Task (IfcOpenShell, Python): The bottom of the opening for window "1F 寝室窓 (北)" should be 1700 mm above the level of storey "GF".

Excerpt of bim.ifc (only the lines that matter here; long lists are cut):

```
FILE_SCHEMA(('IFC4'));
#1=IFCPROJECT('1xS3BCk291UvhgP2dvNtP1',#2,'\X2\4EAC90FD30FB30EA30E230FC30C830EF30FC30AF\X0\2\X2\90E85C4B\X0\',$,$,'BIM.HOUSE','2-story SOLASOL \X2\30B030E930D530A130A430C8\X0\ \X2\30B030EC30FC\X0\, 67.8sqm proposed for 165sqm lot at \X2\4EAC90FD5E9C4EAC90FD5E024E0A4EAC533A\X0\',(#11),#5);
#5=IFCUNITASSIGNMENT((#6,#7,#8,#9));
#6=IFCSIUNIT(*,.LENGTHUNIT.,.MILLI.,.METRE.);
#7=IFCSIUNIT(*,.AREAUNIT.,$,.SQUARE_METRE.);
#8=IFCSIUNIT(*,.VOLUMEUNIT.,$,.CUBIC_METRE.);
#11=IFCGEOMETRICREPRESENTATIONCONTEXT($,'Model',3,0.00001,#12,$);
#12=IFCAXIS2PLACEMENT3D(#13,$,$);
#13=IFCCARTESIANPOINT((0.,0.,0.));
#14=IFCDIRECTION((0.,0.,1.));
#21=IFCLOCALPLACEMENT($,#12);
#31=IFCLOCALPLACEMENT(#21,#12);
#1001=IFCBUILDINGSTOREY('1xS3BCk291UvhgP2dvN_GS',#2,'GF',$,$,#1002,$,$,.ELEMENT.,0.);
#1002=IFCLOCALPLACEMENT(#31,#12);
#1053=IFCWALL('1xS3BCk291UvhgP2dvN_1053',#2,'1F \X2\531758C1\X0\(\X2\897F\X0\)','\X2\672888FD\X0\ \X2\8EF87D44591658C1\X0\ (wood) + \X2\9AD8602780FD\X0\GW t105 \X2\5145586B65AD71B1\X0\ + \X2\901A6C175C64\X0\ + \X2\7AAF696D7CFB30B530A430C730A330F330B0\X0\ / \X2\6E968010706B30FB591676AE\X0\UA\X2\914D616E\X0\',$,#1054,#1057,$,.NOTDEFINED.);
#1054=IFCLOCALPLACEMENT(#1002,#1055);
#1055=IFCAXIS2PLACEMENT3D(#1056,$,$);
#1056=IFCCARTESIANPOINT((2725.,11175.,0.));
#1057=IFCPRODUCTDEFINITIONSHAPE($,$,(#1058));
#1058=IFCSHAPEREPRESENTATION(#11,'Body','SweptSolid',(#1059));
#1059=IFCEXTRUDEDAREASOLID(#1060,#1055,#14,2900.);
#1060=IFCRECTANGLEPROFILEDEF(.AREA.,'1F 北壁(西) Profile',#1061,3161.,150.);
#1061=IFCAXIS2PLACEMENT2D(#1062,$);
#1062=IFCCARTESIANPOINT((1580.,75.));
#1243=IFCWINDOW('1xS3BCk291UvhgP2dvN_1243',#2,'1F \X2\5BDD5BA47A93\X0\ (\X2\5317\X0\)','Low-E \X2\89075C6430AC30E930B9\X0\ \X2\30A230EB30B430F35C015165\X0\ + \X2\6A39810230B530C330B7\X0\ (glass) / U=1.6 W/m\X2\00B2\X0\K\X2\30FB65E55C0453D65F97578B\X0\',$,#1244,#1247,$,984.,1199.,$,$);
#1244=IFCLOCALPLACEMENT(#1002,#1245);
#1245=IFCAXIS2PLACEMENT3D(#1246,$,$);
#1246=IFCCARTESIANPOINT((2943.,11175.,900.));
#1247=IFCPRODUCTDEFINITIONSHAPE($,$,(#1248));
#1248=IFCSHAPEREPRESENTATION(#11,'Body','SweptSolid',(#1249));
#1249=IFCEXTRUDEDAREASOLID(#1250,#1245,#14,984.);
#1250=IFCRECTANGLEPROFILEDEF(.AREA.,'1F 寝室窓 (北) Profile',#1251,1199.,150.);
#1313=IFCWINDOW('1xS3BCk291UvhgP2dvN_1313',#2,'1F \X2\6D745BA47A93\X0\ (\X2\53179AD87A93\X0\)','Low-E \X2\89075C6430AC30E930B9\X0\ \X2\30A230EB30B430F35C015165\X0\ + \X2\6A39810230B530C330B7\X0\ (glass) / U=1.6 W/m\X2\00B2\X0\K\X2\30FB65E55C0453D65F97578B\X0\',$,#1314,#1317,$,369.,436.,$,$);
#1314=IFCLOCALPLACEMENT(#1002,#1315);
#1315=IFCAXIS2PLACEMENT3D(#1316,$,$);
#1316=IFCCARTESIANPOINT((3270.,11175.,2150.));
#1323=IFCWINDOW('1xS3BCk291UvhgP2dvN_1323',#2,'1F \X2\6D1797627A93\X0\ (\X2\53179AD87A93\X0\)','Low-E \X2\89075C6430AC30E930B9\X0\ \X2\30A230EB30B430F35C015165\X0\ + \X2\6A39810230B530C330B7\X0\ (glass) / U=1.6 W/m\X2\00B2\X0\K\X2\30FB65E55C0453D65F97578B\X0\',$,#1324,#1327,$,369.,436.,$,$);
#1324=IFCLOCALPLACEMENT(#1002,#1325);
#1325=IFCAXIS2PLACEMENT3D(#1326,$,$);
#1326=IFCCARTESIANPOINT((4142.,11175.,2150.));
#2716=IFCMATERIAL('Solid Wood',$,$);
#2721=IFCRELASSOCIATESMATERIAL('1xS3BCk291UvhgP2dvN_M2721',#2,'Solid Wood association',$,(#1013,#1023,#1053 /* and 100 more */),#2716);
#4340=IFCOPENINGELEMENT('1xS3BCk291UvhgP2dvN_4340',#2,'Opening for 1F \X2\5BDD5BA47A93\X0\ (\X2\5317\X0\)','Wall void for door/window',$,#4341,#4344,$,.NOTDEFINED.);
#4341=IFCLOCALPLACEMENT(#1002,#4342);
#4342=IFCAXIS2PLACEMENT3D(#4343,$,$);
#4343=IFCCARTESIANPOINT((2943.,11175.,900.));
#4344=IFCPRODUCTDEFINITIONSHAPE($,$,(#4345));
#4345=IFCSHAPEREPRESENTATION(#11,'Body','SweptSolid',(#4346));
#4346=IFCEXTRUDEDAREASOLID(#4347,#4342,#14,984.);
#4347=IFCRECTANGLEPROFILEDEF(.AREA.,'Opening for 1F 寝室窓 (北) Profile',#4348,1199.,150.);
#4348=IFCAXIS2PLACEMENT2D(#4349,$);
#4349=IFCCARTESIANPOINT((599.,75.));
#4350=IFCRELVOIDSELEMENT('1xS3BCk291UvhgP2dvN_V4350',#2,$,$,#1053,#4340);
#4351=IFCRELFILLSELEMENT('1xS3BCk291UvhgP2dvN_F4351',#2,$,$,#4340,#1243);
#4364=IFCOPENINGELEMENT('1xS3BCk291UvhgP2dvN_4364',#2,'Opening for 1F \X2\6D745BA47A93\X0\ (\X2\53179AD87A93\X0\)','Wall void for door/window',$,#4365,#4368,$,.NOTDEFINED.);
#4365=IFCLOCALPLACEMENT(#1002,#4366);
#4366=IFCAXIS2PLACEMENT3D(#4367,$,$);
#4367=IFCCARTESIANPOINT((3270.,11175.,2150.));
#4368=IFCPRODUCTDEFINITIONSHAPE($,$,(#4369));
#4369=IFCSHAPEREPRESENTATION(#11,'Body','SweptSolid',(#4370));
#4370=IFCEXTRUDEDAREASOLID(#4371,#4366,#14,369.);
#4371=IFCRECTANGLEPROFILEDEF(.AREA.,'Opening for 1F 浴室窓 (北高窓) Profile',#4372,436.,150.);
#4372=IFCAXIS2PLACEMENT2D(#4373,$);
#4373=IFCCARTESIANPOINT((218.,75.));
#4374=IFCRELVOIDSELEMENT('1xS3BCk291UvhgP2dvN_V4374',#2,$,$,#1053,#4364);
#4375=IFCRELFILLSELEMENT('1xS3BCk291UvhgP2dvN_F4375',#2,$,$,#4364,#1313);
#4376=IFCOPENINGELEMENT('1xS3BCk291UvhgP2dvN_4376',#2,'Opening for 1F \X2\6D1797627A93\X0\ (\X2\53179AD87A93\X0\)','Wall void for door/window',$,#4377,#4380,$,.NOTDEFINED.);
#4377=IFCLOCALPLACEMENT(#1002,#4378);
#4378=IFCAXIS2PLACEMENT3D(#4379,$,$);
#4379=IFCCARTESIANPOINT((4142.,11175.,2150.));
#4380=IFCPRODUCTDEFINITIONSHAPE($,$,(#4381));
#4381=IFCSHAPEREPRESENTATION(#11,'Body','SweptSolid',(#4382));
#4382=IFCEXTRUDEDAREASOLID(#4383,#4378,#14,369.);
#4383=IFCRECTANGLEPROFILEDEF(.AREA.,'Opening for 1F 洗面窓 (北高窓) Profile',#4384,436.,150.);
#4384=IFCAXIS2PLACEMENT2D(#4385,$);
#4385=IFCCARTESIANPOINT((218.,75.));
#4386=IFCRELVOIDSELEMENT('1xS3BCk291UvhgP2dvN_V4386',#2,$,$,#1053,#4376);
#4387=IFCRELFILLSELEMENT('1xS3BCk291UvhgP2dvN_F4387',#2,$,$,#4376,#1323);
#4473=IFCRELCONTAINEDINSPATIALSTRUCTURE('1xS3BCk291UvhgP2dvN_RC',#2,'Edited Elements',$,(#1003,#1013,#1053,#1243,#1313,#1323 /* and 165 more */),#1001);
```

```python
import numpy as np
import ifcopenshell
import ifcopenshell.api.geometry
import ifcopenshell.geom
import ifcopenshell.util.element
import ifcopenshell.util.placement
import ifcopenshell.util.shape
import ifcopenshell.util.unit

model = ifcopenshell.open("bim.ifc")
unit_scale = ifcopenshell.util.unit.calculate_unit_scale(model)

window = model.by_guid("1xS3BCk291UvhgP2dvN_1243")
opening = window.FillsVoids[0].RelatingOpeningElement
storey = ifcopenshell.util.element.get_container(window, ifc_class="IfcBuildingStorey")
level = ifcopenshell.util.placement.get_local_placement(storey.ObjectPlacement)[2, 3]

# The opening's origin need not be at the sill, so measure its lowest point.
shape = ifcopenshell.geom.create_shape(ifcopenshell.geom.settings(), opening)
bottom = ifcopenshell.util.shape.get_shape_bottom_elevation(shape, shape.geometry) / unit_scale
dz = level + 1.7 / unit_scale - bottom

shift = np.array([0.0, 0.0, dz])
# The window is not placed relative to its opening, so move both.
for product in (opening, window):
    matrix = ifcopenshell.util.placement.get_local_placement(product.ObjectPlacement)
    matrix[:3, 3] += shift
    ifcopenshell.api.geometry.edit_object_placement(model, product=product, matrix=matrix, is_si=False)

print(f"moved by {dz * unit_scale:+.3f} m")

model.write("bim_rev.ifc")
```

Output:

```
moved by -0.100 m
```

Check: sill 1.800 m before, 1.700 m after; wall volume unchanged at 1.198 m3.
